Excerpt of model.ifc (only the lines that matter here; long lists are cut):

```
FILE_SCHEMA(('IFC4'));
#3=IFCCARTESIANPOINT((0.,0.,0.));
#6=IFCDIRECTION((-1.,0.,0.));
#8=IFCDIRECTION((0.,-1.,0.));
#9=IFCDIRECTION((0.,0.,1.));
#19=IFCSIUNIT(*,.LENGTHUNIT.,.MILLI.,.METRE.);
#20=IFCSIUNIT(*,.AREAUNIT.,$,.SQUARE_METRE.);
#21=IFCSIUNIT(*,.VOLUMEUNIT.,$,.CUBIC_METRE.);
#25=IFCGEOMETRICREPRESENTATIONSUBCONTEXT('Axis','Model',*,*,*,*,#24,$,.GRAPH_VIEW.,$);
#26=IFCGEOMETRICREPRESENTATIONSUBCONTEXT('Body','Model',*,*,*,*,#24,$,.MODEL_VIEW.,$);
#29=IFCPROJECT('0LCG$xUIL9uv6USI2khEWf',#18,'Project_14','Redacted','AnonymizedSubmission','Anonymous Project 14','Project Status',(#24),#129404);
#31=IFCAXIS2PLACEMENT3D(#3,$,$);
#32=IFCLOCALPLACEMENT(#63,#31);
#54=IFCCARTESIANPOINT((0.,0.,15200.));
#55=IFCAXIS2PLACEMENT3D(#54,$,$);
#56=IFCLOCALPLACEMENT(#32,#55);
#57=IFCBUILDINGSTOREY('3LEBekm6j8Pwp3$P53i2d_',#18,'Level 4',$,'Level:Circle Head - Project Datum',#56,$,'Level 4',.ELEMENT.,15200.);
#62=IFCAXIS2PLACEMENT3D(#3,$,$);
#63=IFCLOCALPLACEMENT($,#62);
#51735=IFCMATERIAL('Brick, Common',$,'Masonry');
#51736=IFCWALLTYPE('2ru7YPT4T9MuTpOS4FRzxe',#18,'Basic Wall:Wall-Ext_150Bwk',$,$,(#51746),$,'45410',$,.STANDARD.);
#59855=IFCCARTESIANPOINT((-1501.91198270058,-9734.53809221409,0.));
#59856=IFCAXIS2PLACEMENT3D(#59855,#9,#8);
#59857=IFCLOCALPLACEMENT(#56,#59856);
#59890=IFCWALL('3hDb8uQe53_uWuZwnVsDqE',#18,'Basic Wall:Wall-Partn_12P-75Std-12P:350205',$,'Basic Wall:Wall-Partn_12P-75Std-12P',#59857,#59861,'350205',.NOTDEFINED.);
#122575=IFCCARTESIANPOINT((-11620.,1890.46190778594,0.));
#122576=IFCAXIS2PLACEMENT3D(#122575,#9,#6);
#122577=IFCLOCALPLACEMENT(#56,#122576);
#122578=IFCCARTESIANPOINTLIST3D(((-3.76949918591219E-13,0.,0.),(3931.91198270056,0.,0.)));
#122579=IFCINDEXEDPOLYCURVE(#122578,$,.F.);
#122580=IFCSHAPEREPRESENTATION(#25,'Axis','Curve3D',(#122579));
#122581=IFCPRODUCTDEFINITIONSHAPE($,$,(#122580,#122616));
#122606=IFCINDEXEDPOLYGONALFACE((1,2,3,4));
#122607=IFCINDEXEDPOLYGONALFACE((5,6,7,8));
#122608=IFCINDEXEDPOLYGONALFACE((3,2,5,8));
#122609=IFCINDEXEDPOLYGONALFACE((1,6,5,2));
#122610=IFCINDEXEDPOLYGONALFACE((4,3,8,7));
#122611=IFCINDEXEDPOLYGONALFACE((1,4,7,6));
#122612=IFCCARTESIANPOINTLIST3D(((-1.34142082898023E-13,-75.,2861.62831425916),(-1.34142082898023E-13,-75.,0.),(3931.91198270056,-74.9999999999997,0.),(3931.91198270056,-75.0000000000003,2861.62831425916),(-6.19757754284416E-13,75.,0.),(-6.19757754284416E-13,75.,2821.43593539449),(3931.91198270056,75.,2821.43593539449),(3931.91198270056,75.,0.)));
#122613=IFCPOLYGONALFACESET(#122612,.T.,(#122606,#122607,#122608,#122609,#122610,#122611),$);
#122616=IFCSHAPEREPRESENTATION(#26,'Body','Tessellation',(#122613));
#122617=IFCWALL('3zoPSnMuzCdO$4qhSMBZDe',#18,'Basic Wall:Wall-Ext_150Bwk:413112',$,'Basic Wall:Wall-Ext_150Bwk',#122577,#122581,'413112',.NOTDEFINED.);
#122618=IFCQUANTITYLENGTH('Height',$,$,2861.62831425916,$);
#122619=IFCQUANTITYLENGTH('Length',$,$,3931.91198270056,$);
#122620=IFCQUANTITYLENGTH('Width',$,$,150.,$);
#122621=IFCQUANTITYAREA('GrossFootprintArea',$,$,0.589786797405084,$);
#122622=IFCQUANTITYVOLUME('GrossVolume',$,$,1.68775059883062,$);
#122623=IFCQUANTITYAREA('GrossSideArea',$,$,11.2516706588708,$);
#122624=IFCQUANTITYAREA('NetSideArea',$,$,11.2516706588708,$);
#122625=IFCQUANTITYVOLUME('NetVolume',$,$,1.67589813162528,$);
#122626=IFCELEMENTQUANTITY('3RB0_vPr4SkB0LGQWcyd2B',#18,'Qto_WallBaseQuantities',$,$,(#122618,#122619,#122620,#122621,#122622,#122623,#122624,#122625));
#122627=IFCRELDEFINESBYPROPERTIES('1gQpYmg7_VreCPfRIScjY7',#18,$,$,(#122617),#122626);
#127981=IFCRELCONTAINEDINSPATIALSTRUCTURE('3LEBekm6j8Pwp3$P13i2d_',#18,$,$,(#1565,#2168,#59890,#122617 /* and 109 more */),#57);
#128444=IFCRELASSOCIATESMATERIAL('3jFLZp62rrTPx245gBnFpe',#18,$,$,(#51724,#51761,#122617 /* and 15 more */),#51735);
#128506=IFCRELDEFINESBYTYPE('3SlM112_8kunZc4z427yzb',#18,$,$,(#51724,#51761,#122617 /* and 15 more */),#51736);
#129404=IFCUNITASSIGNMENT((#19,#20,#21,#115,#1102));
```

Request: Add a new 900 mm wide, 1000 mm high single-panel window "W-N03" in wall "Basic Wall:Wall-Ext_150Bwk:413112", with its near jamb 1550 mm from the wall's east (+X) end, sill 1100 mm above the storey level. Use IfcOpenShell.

```python
import numpy as np
import ifcopenshell
import ifcopenshell.api.feature
import ifcopenshell.api.geometry
import ifcopenshell.api.pset
import ifcopenshell.api.root
import ifcopenshell.api.spatial
import ifcopenshell.geom
import ifcopenshell.util.element
import ifcopenshell.util.placement
import ifcopenshell.util.representation
import ifcopenshell.util.shape
import ifcopenshell.util.unit

model = ifcopenshell.open("model.ifc")
unit_scale = ifcopenshell.util.unit.calculate_unit_scale(model)
area_scale = ifcopenshell.util.unit.calculate_unit_scale(model, "AREAUNIT")
volume_scale = ifcopenshell.util.unit.calculate_unit_scale(model, "VOLUMEUNIT")
settings = ifcopenshell.geom.settings()


def volume(element):
    """Net volume in cubic metres, openings subtracted."""
    shape = ifcopenshell.geom.create_shape(settings, element)
    return ifcopenshell.util.shape.get_volume(shape.geometry)


wall = model.by_id(122617)
storey = ifcopenshell.util.element.get_container(wall, ifc_class="IfcBuildingStorey")
context = ifcopenshell.util.representation.get_context(model, "Model", "Body", "MODEL_VIEW")
before = volume(wall)

width, height, from_end, sill = 0.9, 1, 1.55, 1.1  # metres

# The wall runs along its own X axis, and the end named is its -X end.
wall_shape = ifcopenshell.geom.create_shape(settings, wall)
x, y, z = ifcopenshell.util.shape.get_vertices(wall_shape.geometry).T
start = x.min() + from_end
face, thickness = float(y.min()), float(y.max() - y.min())
wall_matrix = ifcopenshell.util.placement.get_local_placement(wall.ObjectPlacement)
level = ifcopenshell.util.placement.get_local_placement(storey.ObjectPlacement)[2, 3]


def in_wall(x, y):
    """Placement at x, y metres in the wall's axes, at sill height."""
    matrix = wall_matrix.copy()
    matrix[:, 3] = wall_matrix @ np.array([x / unit_scale, y / unit_scale, 0.0, 1.0])
    matrix[2, 3] = level + sill / unit_scale
    return matrix


# Opening: a box that overshoots both wall faces by 50 mm.
opening = ifcopenshell.api.root.create_entity(model, ifc_class="IfcOpeningElement", predefined_type="OPENING")
box = ifcopenshell.api.geometry.add_wall_representation(
    model, context=context, length=width, height=height, thickness=thickness + 0.1
)
ifcopenshell.api.geometry.assign_representation(model, product=opening, representation=box)
ifcopenshell.api.geometry.edit_object_placement(model, product=opening, matrix=in_wall(start, face - 0.05), is_si=False)
ifcopenshell.api.feature.add_feature(model, feature=opening, element=wall)

window = ifcopenshell.api.root.create_entity(model, ifc_class="IfcWindow", name="W-N03", predefined_type="WINDOW")
window.OverallWidth, window.OverallHeight = width / unit_scale, height / unit_scale
window.PartitioningType = "SINGLE_PANEL"
body = ifcopenshell.api.geometry.add_window_representation(
    model,
    context=context,
    overall_width=window.OverallWidth,
    overall_height=window.OverallHeight,
    partition_type="SINGLE_PANEL",
)
ifcopenshell.api.geometry.assign_representation(model, product=window, representation=body)
ifcopenshell.api.spatial.assign_container(model, products=[window], relating_structure=storey)
ifcopenshell.api.feature.add_filling(model, opening=opening, element=window)

# Centre the window in the wall's thickness.
ifcopenshell.api.geometry.edit_object_placement(model, product=window, matrix=in_wall(start, face), is_si=False)
window_shape = ifcopenshell.geom.create_shape(settings, window)
depth = ifcopenshell.util.shape.get_vertices(window_shape.geometry)[:, 1]
offset = face + thickness / 2 - (depth.min() + depth.max()) / 2
ifcopenshell.api.geometry.edit_object_placement(model, product=window, matrix=in_wall(start, offset), is_si=False)

after = volume(wall)

# Update the wall's stored quantities.
qto = model.by_id(ifcopenshell.util.element.get_pset(wall, "Qto_WallBaseQuantities", should_inherit=False)["id"])
ifcopenshell.api.pset.edit_qto(model, qto=qto, properties={
    "NetSideArea": after / thickness / area_scale,
    "NetVolume": after / volume_scale,
})

print(f"wall volume {before:.3f} -> {after:.3f} m3")

model.write("model_v2.ifc")
```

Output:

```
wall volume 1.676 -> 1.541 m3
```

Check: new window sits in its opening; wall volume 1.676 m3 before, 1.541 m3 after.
